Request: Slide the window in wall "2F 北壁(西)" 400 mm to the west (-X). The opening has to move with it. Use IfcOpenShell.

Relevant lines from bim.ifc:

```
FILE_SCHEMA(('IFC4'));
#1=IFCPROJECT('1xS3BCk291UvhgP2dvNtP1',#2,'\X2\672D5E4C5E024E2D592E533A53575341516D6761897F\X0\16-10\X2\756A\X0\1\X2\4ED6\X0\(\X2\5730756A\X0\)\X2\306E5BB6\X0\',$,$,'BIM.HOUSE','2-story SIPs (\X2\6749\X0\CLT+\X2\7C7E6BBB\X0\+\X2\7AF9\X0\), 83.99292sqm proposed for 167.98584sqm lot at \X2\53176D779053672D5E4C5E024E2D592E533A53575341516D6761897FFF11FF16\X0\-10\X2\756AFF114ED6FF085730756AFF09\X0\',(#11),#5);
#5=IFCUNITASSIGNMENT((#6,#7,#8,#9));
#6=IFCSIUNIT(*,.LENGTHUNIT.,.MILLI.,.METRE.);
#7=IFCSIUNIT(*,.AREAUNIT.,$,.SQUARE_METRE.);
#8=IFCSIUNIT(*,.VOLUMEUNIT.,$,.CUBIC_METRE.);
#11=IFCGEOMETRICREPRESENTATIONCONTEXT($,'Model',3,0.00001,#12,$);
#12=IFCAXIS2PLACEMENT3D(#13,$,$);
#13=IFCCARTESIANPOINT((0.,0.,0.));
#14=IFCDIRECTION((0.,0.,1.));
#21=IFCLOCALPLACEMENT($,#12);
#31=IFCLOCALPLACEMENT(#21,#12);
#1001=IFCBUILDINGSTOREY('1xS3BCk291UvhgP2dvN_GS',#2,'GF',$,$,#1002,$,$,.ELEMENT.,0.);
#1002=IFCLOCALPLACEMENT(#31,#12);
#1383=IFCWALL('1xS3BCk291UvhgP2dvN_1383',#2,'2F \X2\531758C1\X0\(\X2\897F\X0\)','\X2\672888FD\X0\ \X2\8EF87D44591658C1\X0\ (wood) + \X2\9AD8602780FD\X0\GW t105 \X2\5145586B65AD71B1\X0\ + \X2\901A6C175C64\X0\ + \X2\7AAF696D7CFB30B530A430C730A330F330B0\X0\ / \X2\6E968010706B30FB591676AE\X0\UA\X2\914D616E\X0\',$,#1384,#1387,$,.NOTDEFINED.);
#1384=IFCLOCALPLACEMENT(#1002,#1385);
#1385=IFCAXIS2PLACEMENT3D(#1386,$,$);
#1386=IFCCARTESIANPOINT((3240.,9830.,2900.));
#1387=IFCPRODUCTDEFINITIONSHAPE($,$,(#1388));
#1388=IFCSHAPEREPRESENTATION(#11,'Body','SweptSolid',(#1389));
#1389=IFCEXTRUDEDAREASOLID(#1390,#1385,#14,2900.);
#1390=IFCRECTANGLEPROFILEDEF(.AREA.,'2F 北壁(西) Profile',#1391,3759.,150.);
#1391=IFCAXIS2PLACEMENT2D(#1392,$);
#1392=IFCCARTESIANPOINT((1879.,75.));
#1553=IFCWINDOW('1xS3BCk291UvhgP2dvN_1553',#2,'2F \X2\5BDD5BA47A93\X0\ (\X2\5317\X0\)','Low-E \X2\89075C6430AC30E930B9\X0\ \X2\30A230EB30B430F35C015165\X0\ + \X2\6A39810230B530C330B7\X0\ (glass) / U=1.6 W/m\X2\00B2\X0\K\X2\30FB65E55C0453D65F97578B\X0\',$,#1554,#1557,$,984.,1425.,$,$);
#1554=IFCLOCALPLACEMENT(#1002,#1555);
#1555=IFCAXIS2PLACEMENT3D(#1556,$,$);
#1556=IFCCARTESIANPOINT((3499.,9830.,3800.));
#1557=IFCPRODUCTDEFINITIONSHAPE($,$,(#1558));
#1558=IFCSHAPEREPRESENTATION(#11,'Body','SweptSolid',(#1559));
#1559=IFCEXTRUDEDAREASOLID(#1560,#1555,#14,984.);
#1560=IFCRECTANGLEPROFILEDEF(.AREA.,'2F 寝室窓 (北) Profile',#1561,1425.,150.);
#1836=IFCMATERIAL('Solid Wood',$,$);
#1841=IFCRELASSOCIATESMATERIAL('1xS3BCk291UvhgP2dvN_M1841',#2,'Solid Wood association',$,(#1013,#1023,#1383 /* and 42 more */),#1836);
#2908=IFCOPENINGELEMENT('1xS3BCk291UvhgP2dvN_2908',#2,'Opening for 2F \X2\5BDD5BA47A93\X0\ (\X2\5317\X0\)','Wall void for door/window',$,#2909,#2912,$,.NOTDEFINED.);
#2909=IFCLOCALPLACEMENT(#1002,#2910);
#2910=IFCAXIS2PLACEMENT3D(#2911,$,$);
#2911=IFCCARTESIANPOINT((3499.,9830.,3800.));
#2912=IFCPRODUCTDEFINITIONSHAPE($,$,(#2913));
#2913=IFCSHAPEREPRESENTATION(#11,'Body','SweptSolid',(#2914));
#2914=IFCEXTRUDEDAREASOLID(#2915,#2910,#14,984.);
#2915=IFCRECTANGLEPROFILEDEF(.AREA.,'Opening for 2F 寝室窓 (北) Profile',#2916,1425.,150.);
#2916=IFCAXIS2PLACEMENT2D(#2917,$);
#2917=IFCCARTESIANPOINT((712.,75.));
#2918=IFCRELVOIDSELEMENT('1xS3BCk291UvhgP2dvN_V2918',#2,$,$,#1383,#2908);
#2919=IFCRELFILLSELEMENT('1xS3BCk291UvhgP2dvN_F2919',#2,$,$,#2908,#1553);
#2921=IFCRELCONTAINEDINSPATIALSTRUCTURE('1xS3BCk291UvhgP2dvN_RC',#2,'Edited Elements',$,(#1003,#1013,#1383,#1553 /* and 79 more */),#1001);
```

```python
import ifcopenshell
import ifcopenshell.api.geometry
import ifcopenshell.util.placement

model = ifcopenshell.open("bim.ifc")

window = model.by_id(1553)
opening = window.FillsVoids[0].RelatingOpeningElement
wall = opening.VoidsElements[0].RelatingBuildingElement

wall_matrix = ifcopenshell.util.placement.get_local_placement(wall.ObjectPlacement)
shift = wall_matrix[:3, 0] * -400.0
before = ifcopenshell.util.placement.get_local_placement(window.ObjectPlacement)[:3, 3].copy()

# The window is not placed relative to its opening, so move both.
for product in (opening, window):
    matrix = ifcopenshell.util.placement.get_local_placement(product.ObjectPlacement)
    matrix[:3, 3] += shift
    ifcopenshell.api.geometry.edit_object_placement(model, product=product, matrix=matrix, is_si=False)

after = ifcopenshell.util.placement.get_local_placement(window.ObjectPlacement)[:3, 3]
print("window moved by", (after - before).round(3) + 0.0)

model.write("bim_v2.ifc")
```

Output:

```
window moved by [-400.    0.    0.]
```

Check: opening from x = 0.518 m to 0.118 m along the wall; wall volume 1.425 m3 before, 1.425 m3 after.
